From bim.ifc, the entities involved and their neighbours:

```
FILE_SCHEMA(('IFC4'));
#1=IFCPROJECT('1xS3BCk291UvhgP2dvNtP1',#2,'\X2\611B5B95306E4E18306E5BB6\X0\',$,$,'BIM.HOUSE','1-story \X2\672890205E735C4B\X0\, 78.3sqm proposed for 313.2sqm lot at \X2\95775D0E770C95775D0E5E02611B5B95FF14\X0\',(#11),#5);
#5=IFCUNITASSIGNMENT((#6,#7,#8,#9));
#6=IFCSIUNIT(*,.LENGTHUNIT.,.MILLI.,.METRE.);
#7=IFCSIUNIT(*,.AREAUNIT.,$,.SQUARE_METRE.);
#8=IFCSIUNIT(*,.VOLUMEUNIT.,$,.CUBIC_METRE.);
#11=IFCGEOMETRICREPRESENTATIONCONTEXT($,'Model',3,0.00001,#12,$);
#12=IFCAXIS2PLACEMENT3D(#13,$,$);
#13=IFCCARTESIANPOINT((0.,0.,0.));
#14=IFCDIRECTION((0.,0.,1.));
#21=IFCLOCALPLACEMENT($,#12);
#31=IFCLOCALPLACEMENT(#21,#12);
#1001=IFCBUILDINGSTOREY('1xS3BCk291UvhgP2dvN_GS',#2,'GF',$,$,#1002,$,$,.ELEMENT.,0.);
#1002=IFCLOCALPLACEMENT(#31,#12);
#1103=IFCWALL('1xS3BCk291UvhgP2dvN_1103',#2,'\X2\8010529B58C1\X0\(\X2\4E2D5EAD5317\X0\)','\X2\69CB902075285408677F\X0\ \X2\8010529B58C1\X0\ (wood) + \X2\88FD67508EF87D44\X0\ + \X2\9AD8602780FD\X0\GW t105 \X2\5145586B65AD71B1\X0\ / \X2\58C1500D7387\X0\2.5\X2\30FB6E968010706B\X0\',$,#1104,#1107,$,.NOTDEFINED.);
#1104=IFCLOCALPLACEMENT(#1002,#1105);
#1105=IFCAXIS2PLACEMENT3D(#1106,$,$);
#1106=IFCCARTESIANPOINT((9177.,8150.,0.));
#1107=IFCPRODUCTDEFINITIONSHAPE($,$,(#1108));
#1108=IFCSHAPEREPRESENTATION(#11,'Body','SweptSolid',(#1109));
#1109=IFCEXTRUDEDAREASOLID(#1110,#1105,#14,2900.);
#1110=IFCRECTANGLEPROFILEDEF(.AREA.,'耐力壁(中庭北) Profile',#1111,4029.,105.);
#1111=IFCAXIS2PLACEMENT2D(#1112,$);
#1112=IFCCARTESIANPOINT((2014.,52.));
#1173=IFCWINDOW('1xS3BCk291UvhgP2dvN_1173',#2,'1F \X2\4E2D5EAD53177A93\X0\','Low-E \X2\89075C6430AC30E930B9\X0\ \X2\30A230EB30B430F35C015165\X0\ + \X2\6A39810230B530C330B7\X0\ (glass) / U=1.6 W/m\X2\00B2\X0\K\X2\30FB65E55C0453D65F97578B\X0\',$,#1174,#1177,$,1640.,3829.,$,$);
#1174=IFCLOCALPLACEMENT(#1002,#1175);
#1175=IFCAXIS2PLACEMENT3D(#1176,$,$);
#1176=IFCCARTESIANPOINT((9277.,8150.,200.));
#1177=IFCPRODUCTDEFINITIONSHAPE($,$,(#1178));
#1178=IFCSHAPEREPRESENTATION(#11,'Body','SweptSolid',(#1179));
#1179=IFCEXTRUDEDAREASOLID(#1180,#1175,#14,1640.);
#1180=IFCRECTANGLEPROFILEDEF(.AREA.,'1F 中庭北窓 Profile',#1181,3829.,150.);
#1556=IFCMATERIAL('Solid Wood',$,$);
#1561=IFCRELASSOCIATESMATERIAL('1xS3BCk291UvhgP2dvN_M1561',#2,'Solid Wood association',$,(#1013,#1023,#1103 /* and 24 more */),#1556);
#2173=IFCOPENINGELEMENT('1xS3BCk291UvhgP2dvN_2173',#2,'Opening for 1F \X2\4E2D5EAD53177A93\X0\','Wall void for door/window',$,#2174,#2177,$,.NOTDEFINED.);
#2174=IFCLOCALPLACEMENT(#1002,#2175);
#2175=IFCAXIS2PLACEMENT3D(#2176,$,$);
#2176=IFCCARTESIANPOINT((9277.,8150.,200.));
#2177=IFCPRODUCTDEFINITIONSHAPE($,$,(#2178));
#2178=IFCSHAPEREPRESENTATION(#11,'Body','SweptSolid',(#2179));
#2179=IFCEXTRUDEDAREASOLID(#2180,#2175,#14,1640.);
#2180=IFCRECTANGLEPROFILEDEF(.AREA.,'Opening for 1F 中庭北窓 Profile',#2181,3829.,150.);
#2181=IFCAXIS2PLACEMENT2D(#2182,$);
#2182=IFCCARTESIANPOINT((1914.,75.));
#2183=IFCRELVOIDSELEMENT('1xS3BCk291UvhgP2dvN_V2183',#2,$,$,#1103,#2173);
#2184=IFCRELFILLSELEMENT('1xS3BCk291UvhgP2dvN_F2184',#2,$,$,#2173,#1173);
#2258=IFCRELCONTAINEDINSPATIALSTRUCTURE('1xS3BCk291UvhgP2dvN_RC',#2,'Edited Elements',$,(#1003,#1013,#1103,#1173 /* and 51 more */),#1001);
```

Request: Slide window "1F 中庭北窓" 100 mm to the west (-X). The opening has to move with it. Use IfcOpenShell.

```python
import ifcopenshell
import ifcopenshell.api.geometry
import ifcopenshell.util.placement

model = ifcopenshell.open("bim.ifc")

window = model.by_guid("1xS3BCk291UvhgP2dvN_1173")
opening = window.FillsVoids[0].RelatingOpeningElement
wall = opening.VoidsElements[0].RelatingBuildingElement

wall_matrix = ifcopenshell.util.placement.get_local_placement(wall.ObjectPlacement)
shift = wall_matrix[:3, 0] * -100.0
before = ifcopenshell.util.placement.get_local_placement(window.ObjectPlacement)[:3, 3].copy()

# The window is not placed relative to its opening, so move both.
for product in (opening, window):
    matrix = ifcopenshell.util.placement.get_local_placement(product.ObjectPlacement)
    matrix[:3, 3] += shift
    ifcopenshell.api.geometry.edit_object_placement(model, product=product, matrix=matrix, is_si=False)

after = ifcopenshell.util.placement.get_local_placement(window.ObjectPlacement)[:3, 3]
print("window moved by", (after - before).round(3) + 0.0)

model.write("bim_updated.ifc")
```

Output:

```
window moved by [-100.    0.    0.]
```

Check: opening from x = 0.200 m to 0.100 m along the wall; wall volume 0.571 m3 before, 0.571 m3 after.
